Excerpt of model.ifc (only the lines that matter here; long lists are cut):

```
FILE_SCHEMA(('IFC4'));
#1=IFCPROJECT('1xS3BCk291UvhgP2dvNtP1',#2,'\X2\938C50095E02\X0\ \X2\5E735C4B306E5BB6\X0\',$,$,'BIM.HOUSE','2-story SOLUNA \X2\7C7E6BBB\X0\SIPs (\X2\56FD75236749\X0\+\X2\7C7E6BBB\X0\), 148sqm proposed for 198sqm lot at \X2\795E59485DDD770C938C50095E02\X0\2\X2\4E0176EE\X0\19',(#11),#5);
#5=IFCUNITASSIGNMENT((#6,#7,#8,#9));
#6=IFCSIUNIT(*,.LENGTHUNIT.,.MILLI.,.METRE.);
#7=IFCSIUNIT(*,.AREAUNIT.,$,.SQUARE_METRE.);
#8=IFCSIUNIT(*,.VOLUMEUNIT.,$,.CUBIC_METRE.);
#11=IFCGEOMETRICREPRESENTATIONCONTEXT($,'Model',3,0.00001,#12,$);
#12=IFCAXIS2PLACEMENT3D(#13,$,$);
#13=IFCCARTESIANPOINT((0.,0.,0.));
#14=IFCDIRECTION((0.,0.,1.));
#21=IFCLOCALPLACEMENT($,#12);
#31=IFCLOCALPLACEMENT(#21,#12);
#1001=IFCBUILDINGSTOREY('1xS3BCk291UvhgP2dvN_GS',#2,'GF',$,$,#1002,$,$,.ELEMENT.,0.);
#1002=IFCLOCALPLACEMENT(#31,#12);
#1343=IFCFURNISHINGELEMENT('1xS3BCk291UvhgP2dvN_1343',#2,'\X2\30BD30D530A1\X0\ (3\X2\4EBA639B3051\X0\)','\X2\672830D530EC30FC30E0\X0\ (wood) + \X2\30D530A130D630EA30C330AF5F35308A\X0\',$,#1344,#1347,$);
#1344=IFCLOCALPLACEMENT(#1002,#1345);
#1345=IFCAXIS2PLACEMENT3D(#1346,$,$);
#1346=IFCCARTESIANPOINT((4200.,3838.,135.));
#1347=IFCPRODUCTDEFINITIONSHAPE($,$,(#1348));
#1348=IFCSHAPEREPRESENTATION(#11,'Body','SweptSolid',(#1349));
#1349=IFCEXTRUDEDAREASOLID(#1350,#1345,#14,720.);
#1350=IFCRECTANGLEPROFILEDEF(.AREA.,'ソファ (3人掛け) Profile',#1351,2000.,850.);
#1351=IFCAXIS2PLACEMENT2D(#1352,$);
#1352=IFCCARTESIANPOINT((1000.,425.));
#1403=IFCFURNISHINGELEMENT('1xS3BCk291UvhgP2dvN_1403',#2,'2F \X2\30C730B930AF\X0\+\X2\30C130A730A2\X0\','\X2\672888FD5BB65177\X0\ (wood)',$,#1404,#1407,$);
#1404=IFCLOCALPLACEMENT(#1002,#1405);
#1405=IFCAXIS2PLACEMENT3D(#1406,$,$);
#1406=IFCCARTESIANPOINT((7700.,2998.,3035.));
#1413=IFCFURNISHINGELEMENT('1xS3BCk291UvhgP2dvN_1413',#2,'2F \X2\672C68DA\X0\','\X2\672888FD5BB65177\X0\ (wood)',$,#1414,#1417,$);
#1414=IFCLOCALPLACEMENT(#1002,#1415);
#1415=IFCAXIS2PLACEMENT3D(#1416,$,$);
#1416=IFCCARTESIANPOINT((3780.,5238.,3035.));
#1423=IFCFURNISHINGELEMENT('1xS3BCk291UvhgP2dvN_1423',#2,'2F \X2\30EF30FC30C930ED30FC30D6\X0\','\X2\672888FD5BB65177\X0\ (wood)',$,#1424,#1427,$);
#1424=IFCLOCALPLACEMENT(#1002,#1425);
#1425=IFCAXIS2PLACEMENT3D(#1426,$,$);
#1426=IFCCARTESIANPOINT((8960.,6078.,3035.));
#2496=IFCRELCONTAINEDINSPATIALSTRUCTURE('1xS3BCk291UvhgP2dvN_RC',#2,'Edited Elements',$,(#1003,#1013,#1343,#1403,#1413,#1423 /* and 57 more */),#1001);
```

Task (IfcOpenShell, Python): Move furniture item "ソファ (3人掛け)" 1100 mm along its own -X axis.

```python
import ifcopenshell
import ifcopenshell.api.geometry
import ifcopenshell.util.placement
import ifcopenshell.util.unit

model = ifcopenshell.open("model.ifc")
unit_scale = ifcopenshell.util.unit.calculate_unit_scale(model)

item = model.by_guid("1xS3BCk291UvhgP2dvN_1343")
matrix = ifcopenshell.util.placement.get_local_placement(item.ObjectPlacement)
matrix[:3, 3] -= matrix[:3, 0] * 1.1 / unit_scale
ifcopenshell.api.geometry.edit_object_placement(model, product=item, matrix=matrix, is_si=False)

print(ifcopenshell.util.placement.get_local_placement(item.ObjectPlacement).round(3) + 0.0)

model.write("model-out.ifc")
```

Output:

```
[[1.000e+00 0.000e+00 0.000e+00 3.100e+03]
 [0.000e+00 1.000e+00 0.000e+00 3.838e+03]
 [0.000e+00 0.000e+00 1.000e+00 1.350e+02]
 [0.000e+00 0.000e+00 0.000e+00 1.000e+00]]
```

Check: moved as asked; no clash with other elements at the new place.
